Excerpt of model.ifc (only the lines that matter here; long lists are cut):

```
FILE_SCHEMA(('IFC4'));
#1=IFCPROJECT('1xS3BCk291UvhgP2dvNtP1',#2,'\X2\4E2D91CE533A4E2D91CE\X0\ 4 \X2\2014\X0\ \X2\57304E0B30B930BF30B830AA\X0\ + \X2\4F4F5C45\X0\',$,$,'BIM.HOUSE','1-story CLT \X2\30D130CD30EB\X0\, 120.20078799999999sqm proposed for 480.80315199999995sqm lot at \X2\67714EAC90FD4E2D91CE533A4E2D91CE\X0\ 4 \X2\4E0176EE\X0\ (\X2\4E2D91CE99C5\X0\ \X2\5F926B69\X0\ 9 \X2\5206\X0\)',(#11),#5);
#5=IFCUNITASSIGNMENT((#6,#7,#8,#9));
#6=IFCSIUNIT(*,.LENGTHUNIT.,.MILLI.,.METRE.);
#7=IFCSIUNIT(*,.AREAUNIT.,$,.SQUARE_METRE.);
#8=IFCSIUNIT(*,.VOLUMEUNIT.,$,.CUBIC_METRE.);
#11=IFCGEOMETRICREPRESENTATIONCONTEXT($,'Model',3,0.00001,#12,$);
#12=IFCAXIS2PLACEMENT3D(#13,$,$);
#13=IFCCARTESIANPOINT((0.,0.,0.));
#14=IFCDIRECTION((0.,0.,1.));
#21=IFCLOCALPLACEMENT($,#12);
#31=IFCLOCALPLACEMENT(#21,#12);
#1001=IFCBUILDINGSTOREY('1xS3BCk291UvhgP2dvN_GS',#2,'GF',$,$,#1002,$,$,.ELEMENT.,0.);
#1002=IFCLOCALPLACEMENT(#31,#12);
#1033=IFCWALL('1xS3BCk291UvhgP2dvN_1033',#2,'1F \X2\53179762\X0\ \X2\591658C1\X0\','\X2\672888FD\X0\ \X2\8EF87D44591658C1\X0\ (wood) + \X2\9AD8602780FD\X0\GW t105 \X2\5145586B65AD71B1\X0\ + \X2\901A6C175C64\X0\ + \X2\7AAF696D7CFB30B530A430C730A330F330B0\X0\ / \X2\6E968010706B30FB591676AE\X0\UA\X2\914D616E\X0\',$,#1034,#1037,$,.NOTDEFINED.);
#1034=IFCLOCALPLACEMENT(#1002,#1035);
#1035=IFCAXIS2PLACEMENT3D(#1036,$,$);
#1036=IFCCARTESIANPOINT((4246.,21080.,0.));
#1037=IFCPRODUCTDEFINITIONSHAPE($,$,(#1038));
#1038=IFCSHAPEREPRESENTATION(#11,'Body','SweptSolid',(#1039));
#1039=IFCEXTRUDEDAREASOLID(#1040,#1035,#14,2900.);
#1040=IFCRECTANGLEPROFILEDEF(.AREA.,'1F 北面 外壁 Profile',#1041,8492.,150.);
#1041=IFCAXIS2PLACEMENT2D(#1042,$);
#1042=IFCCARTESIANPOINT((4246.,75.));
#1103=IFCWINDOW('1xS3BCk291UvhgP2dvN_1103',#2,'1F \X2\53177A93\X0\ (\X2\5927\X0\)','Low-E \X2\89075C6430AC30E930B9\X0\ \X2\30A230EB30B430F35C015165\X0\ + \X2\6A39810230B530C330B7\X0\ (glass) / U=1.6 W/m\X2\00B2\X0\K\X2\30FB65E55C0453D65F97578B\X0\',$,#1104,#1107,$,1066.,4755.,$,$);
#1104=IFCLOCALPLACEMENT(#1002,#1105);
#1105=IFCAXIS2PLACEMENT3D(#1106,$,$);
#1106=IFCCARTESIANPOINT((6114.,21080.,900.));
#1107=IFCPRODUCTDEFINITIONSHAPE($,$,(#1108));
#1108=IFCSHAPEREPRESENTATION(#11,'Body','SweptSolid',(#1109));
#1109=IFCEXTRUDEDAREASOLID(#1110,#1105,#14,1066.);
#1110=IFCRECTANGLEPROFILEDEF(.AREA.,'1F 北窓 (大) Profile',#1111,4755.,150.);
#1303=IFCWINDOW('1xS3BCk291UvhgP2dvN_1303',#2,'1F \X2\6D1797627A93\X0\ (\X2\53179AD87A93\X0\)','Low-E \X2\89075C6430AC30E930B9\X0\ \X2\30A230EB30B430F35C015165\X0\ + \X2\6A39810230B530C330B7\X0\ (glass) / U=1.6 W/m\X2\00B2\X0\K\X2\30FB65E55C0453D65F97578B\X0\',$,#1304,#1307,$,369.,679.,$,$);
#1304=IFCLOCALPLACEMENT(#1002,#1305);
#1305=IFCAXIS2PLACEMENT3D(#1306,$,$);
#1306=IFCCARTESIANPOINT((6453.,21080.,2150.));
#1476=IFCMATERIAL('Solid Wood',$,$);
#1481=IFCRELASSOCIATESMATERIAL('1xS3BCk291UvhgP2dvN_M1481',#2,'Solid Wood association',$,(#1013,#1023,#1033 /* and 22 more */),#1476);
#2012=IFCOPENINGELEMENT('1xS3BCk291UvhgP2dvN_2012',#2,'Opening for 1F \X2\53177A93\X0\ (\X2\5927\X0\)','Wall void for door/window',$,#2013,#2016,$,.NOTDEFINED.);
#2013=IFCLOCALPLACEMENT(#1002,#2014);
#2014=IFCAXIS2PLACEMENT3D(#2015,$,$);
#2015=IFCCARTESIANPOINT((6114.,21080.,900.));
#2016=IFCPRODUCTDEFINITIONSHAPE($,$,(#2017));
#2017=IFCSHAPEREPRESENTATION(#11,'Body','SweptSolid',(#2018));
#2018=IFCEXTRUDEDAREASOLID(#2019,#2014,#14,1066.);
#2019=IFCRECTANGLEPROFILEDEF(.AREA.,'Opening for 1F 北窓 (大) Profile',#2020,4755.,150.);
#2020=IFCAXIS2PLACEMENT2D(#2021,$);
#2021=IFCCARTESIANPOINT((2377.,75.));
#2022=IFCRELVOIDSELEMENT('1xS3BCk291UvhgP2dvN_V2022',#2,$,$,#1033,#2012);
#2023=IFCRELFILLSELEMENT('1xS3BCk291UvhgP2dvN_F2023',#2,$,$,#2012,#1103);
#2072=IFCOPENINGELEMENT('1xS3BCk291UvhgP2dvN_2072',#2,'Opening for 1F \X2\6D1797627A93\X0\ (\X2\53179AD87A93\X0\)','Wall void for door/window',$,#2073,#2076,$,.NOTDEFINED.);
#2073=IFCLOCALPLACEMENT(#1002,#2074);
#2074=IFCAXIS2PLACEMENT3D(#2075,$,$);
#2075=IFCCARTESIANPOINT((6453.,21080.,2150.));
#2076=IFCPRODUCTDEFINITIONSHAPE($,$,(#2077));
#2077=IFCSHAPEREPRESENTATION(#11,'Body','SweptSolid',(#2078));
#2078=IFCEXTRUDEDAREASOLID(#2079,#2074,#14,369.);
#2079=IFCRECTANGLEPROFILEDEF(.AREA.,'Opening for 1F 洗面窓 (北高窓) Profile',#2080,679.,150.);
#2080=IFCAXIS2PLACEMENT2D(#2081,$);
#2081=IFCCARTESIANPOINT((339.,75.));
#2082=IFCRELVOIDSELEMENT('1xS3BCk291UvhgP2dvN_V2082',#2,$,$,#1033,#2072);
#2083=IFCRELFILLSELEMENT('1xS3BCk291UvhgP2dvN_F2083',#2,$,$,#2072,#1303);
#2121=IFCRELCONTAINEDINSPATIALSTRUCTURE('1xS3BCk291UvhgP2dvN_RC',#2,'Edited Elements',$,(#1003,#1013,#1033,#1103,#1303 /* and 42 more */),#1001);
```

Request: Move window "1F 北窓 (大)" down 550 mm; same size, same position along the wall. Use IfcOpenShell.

```python
import numpy as np
import ifcopenshell
import ifcopenshell.api.geometry
import ifcopenshell.util.placement
import ifcopenshell.util.unit

model = ifcopenshell.open("model.ifc")
unit_scale = ifcopenshell.util.unit.calculate_unit_scale(model)

window = model.by_guid("1xS3BCk291UvhgP2dvN_1103")
opening = window.FillsVoids[0].RelatingOpeningElement
dz = -550.0

shift = np.array([0.0, 0.0, dz])
# The window is not placed relative to its opening, so move both.
for product in (opening, window):
    matrix = ifcopenshell.util.placement.get_local_placement(product.ObjectPlacement)
    matrix[:3, 3] += shift
    ifcopenshell.api.geometry.edit_object_placement(model, product=product, matrix=matrix, is_si=False)

print(f"moved by {dz * unit_scale:+.3f} m")

model.write("model_v2.ifc")
```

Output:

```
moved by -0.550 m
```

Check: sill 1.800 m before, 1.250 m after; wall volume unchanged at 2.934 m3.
